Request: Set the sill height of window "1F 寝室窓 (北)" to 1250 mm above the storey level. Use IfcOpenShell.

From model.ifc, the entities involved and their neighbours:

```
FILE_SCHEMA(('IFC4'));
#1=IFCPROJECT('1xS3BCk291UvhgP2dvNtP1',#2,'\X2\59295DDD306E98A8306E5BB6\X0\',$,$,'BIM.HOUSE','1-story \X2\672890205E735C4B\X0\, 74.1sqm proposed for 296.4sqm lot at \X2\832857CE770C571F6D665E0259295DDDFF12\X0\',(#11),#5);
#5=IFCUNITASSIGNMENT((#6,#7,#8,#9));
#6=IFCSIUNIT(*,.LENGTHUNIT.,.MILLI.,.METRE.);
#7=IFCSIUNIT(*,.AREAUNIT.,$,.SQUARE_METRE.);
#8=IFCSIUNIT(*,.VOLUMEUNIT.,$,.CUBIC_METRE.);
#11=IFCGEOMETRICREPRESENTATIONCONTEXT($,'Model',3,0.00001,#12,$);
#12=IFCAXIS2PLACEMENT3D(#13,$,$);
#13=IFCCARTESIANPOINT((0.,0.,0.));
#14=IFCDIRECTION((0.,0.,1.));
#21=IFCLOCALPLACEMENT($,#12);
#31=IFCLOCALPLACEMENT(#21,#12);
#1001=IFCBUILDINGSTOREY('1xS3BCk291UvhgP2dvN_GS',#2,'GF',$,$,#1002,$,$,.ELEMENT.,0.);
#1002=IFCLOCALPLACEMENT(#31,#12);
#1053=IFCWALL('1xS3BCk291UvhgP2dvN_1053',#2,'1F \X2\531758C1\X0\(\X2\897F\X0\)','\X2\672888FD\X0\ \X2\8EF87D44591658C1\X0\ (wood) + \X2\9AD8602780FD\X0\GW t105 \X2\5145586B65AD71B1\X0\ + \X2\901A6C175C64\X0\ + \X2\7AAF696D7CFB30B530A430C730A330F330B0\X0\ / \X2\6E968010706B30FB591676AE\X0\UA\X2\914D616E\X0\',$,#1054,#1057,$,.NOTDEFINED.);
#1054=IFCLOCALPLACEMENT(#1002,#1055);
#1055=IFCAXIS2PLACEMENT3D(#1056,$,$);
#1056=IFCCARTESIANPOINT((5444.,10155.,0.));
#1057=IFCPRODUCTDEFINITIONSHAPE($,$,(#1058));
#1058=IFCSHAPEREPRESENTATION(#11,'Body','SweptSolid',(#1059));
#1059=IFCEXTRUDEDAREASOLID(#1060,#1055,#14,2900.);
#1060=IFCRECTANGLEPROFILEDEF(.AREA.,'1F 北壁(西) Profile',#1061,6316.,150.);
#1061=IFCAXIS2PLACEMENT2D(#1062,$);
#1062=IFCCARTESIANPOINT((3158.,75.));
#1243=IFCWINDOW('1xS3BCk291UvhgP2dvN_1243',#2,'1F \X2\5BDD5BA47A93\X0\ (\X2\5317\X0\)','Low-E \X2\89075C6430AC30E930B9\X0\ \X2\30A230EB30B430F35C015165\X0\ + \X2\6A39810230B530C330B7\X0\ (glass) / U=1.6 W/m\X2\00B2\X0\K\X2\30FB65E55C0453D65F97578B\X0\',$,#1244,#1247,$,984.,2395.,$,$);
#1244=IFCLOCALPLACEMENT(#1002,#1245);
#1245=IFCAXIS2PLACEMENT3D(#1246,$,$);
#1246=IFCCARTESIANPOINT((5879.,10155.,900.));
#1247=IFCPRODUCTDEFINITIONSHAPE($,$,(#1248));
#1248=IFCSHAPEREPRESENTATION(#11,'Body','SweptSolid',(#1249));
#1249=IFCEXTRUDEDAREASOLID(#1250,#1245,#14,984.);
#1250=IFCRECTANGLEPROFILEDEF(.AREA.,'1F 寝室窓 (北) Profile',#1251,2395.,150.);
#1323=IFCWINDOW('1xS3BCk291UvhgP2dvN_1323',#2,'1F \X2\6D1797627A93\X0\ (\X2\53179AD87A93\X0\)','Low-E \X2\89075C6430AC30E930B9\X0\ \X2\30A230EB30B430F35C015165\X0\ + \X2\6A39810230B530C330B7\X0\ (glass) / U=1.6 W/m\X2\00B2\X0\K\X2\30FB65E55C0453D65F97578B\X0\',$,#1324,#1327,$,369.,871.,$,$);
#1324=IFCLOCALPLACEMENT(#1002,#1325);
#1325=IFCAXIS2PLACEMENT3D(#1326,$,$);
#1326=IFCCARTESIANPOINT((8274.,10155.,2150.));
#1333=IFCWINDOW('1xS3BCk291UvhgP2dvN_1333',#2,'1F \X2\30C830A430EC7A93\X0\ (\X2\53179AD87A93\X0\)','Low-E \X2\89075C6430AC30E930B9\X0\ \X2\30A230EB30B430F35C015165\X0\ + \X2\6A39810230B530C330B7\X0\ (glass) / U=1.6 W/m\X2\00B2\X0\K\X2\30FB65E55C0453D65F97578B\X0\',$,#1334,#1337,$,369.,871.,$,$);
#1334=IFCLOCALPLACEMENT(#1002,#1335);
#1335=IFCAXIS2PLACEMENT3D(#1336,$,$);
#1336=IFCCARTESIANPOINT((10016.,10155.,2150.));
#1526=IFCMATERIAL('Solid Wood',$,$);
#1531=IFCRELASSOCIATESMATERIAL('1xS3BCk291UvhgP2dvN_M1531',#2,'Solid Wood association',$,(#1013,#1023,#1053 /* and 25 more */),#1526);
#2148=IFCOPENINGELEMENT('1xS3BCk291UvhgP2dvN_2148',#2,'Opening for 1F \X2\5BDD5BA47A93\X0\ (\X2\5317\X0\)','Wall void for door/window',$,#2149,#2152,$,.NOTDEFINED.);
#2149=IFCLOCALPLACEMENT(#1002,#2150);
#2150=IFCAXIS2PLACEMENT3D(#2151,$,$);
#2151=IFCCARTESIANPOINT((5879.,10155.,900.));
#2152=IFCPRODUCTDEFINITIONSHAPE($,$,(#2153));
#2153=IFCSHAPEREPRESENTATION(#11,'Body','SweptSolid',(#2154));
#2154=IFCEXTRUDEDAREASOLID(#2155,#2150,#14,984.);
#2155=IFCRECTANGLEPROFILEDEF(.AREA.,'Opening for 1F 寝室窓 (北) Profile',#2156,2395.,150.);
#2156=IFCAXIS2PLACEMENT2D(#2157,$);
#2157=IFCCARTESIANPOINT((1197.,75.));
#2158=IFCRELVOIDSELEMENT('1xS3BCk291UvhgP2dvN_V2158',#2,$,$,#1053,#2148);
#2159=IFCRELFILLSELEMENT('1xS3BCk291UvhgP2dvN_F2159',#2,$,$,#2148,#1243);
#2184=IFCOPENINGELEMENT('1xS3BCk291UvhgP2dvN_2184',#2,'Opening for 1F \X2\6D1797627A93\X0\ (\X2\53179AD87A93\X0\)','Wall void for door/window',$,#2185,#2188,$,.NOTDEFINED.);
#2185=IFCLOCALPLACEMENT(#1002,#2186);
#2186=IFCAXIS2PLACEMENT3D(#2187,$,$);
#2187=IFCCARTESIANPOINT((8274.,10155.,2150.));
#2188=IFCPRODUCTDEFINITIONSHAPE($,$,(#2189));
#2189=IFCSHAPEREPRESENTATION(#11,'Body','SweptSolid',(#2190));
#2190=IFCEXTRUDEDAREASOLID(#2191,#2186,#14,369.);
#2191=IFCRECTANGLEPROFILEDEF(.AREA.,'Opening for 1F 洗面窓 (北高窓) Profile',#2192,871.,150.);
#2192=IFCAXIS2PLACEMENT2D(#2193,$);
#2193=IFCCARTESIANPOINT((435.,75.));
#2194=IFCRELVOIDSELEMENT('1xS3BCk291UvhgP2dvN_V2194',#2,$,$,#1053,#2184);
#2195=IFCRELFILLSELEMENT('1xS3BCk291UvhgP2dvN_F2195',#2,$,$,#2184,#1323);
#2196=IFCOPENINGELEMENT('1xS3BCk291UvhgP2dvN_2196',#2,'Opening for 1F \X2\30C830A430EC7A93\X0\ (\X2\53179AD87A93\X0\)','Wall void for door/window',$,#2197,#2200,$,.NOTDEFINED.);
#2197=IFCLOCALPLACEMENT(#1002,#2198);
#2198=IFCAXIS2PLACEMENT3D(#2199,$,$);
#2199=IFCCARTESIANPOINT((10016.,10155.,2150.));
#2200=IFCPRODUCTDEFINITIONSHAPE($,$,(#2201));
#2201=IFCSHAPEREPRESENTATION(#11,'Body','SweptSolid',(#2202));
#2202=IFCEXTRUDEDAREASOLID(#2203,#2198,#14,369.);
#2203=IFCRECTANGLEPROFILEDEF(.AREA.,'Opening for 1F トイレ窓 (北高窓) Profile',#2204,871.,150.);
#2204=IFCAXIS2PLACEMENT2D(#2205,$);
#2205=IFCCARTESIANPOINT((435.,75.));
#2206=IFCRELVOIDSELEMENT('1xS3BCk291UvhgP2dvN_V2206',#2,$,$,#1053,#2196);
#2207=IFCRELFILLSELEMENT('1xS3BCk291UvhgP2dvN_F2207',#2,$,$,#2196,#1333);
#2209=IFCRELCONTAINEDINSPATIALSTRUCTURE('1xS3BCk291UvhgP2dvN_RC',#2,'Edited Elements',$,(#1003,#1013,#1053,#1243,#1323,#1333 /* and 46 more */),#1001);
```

```python
import numpy as np
import ifcopenshell
import ifcopenshell.api.geometry
import ifcopenshell.geom
import ifcopenshell.util.element
import ifcopenshell.util.placement
import ifcopenshell.util.shape
import ifcopenshell.util.unit

model = ifcopenshell.open("model.ifc")
unit_scale = ifcopenshell.util.unit.calculate_unit_scale(model)

window = model.by_id(1243)
opening = window.FillsVoids[0].RelatingOpeningElement
storey = ifcopenshell.util.element.get_container(window, ifc_class="IfcBuildingStorey")
level = ifcopenshell.util.placement.get_local_placement(storey.ObjectPlacement)[2, 3]

# The opening's origin need not be at the sill, so measure its lowest point.
shape = ifcopenshell.geom.create_shape(ifcopenshell.geom.settings(), opening)
bottom = ifcopenshell.util.shape.get_shape_bottom_elevation(shape, shape.geometry) / unit_scale
dz = level + 1.25 / unit_scale - bottom

shift = np.array([0.0, 0.0, dz])
# The window is not placed relative to its opening, so move both.
for product in (opening, window):
    matrix = ifcopenshell.util.placement.get_local_placement(product.ObjectPlacement)
    matrix[:3, 3] += shift
    ifcopenshell.api.geometry.edit_object_placement(model, product=product, matrix=matrix, is_si=False)

print(f"moved by {dz * unit_scale:+.3f} m")

model.write("model_edited.ifc")
```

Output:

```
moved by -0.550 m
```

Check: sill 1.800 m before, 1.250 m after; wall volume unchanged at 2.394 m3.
